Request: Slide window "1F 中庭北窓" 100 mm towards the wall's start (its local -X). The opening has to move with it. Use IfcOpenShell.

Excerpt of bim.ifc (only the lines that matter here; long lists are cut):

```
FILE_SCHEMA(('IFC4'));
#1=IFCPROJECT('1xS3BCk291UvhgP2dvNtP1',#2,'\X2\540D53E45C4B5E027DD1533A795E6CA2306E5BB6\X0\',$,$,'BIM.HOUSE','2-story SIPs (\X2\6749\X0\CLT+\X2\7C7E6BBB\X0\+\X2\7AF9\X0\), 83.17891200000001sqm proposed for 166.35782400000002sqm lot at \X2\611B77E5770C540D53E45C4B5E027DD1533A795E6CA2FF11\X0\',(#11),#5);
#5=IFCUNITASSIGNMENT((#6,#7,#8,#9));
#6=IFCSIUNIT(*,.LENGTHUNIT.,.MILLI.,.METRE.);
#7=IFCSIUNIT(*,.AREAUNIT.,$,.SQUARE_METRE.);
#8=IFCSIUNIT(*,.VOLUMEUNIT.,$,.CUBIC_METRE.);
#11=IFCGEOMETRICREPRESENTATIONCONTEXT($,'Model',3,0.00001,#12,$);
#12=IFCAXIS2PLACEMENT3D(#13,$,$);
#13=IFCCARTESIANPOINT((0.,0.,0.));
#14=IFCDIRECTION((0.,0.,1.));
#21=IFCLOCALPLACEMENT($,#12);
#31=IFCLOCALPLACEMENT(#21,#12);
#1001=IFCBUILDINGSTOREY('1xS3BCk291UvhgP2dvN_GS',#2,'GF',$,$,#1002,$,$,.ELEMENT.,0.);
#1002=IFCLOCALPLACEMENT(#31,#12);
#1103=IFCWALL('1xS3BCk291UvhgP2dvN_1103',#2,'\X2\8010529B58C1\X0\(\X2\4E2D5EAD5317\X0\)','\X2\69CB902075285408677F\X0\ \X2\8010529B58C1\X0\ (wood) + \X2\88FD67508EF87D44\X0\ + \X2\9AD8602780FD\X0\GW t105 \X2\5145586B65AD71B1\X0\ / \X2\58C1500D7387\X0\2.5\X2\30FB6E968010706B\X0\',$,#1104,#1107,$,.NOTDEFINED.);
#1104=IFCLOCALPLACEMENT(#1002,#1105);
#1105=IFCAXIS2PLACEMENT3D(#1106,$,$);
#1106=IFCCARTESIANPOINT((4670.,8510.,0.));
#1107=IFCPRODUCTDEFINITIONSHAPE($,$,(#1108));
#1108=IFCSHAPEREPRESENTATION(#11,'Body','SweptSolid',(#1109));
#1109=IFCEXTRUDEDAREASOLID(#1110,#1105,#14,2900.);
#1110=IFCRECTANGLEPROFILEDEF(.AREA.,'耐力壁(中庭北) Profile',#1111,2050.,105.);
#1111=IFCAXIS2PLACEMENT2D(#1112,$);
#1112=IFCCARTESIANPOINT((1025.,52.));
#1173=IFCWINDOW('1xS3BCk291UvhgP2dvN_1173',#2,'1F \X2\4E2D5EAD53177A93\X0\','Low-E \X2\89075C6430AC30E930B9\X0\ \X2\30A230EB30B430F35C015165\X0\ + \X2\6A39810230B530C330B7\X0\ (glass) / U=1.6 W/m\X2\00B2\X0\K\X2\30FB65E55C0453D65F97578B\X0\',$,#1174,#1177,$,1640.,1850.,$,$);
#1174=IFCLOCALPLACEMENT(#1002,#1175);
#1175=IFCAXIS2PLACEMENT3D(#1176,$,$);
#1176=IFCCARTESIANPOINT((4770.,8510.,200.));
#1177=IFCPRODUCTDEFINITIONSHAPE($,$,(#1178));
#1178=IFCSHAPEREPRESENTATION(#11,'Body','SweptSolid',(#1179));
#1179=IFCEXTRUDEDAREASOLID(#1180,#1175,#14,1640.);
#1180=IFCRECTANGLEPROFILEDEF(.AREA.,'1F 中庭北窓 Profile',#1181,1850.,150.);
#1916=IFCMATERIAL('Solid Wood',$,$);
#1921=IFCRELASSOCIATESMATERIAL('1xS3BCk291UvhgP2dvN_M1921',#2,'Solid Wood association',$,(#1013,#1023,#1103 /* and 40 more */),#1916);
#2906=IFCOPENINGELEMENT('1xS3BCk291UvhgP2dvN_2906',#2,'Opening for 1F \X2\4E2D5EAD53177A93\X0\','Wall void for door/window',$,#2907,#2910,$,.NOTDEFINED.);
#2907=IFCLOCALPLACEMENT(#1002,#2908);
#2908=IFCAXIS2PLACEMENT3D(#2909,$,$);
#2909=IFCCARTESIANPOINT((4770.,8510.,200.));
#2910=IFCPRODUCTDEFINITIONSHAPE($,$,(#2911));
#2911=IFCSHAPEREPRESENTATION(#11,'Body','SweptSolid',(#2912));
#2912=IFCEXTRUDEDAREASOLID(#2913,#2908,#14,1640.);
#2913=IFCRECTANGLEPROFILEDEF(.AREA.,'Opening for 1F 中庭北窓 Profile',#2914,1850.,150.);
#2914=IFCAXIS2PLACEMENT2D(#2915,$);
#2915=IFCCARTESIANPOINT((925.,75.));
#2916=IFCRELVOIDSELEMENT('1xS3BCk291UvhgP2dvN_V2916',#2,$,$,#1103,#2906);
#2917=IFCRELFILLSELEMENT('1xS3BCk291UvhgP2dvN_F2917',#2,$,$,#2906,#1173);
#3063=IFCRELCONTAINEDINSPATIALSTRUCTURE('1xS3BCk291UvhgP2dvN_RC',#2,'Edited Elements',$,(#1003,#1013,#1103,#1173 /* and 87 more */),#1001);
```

```python
import ifcopenshell
import ifcopenshell.api.geometry
import ifcopenshell.util.placement
import ifcopenshell.util.unit

model = ifcopenshell.open("bim.ifc")
unit_scale = ifcopenshell.util.unit.calculate_unit_scale(model)

window = model.by_guid("1xS3BCk291UvhgP2dvN_1173")
opening = window.FillsVoids[0].RelatingOpeningElement
wall = opening.VoidsElements[0].RelatingBuildingElement

wall_matrix = ifcopenshell.util.placement.get_local_placement(wall.ObjectPlacement)
shift = wall_matrix[:3, 0] * -0.1 / unit_scale
before = ifcopenshell.util.placement.get_local_placement(window.ObjectPlacement)[:3, 3].copy()

# The window is not placed relative to its opening, so move both.
for product in (opening, window):
    matrix = ifcopenshell.util.placement.get_local_placement(product.ObjectPlacement)
    matrix[:3, 3] += shift
    ifcopenshell.api.geometry.edit_object_placement(model, product=product, matrix=matrix, is_si=False)

after = ifcopenshell.util.placement.get_local_placement(window.ObjectPlacement)[:3, 3]
print("window moved by", (after - before).round(3) + 0.0)

model.write("bim_updated.ifc")
```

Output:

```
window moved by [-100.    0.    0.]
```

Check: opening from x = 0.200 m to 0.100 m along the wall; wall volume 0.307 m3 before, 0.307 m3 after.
